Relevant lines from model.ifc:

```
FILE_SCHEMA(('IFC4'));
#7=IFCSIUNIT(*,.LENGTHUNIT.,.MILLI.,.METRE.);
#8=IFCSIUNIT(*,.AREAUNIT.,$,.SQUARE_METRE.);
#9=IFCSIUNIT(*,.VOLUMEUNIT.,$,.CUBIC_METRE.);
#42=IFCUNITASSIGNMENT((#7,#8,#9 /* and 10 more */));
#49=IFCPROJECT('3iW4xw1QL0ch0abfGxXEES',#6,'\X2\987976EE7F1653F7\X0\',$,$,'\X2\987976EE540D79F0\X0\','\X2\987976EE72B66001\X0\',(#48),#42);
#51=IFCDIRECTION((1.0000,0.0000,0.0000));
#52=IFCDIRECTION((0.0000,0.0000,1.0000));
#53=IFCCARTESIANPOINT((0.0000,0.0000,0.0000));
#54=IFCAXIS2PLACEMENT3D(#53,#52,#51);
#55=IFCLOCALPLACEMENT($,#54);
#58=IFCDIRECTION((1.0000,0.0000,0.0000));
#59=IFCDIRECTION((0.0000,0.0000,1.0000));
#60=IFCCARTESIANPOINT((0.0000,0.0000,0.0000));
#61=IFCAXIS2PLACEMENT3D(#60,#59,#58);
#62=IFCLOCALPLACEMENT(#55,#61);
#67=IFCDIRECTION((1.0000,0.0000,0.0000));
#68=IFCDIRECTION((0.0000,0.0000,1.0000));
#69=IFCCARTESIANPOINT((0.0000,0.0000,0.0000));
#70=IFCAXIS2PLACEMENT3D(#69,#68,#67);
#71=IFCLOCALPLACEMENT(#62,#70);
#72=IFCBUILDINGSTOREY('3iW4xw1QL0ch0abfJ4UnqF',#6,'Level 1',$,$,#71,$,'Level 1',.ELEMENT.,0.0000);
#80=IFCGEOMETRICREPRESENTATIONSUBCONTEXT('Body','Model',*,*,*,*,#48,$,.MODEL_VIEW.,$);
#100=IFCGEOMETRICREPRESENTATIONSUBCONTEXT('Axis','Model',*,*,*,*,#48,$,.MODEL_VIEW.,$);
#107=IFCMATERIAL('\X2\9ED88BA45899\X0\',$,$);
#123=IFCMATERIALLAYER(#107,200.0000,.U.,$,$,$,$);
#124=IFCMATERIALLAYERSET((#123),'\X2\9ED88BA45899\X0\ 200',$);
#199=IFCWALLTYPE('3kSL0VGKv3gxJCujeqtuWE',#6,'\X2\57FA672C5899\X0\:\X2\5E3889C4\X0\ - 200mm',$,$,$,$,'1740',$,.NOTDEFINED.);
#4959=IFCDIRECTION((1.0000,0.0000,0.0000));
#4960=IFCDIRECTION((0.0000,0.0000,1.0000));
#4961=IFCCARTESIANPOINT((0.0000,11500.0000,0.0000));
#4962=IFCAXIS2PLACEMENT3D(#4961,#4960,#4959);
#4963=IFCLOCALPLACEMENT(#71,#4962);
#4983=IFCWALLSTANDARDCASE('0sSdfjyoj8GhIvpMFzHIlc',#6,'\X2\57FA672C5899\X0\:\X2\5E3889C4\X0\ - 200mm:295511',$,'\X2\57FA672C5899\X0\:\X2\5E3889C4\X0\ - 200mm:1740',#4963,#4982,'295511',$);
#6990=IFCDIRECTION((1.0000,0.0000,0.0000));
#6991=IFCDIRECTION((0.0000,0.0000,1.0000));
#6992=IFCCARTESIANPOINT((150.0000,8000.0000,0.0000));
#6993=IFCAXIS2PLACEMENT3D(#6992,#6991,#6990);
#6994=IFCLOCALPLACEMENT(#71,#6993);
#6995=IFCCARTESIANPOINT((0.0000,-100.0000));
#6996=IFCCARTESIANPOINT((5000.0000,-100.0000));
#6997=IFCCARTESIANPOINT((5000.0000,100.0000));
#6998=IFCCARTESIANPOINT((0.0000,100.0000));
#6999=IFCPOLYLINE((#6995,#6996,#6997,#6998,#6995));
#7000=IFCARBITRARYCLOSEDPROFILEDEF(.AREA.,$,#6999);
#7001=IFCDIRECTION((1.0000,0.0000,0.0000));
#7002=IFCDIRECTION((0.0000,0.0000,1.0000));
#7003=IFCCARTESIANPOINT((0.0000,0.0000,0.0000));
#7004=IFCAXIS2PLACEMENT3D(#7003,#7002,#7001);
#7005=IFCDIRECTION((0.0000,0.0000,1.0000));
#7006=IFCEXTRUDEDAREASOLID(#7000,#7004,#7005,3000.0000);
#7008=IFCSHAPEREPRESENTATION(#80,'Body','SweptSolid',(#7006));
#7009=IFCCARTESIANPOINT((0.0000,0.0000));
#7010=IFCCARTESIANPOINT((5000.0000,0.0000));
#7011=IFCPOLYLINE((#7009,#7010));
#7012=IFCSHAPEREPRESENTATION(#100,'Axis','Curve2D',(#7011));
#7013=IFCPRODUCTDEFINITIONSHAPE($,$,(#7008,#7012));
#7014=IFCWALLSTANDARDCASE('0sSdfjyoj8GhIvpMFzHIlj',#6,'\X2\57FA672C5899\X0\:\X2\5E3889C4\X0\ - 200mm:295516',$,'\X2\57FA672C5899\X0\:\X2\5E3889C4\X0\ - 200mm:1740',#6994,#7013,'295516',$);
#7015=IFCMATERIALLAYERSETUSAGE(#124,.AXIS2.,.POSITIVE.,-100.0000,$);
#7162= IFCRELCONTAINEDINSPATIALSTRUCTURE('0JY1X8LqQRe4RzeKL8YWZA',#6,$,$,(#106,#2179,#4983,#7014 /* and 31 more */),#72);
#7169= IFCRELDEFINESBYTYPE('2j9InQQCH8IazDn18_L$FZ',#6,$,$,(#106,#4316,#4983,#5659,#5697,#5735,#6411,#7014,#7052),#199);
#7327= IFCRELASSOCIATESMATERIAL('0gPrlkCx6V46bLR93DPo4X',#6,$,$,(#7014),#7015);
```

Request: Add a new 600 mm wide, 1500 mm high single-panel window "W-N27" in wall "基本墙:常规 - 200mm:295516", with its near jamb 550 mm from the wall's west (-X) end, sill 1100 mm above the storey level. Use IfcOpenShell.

```python
import numpy as np
import ifcopenshell
import ifcopenshell.api.feature
import ifcopenshell.api.geometry
import ifcopenshell.api.root
import ifcopenshell.api.spatial
import ifcopenshell.geom
import ifcopenshell.util.element
import ifcopenshell.util.placement
import ifcopenshell.util.representation
import ifcopenshell.util.shape
import ifcopenshell.util.unit

model = ifcopenshell.open("model.ifc")
unit_scale = ifcopenshell.util.unit.calculate_unit_scale(model)
settings = ifcopenshell.geom.settings()


def volume(element):
    """Net volume in cubic metres, openings subtracted."""
    shape = ifcopenshell.geom.create_shape(settings, element)
    return ifcopenshell.util.shape.get_volume(shape.geometry)


wall = model.by_id(7014)
storey = ifcopenshell.util.element.get_container(wall, ifc_class="IfcBuildingStorey")
context = ifcopenshell.util.representation.get_context(model, "Model", "Body", "MODEL_VIEW")
before = volume(wall)

width, height, from_end, sill = 0.6, 1.5, 0.55, 1.1  # metres

# The wall runs along its own X axis, and the end named is its -X end.
wall_shape = ifcopenshell.geom.create_shape(settings, wall)
x, y, z = ifcopenshell.util.shape.get_vertices(wall_shape.geometry).T
start = x.min() + from_end
face, thickness = float(y.min()), float(y.max() - y.min())
wall_matrix = ifcopenshell.util.placement.get_local_placement(wall.ObjectPlacement)
level = ifcopenshell.util.placement.get_local_placement(storey.ObjectPlacement)[2, 3]


def in_wall(x, y):
    """Placement at x, y metres in the wall's axes, at sill height."""
    matrix = wall_matrix.copy()
    matrix[:, 3] = wall_matrix @ np.array([x / unit_scale, y / unit_scale, 0.0, 1.0])
    matrix[2, 3] = level + sill / unit_scale
    return matrix


# Opening: a box that overshoots both wall faces by 50 mm.
opening = ifcopenshell.api.root.create_entity(model, ifc_class="IfcOpeningElement", predefined_type="OPENING")
box = ifcopenshell.api.geometry.add_wall_representation(
    model, context=context, length=width, height=height, thickness=thickness + 0.1
)
ifcopenshell.api.geometry.assign_representation(model, product=opening, representation=box)
ifcopenshell.api.geometry.edit_object_placement(model, product=opening, matrix=in_wall(start, face - 0.05), is_si=False)
ifcopenshell.api.feature.add_feature(model, feature=opening, element=wall)

window = ifcopenshell.api.root.create_entity(model, ifc_class="IfcWindow", name="W-N27", predefined_type="WINDOW")
window.OverallWidth, window.OverallHeight = width / unit_scale, height / unit_scale
window.PartitioningType = "SINGLE_PANEL"
body = ifcopenshell.api.geometry.add_window_representation(
    model,
    context=context,
    overall_width=window.OverallWidth,
    overall_height=window.OverallHeight,
    partition_type="SINGLE_PANEL",
)
ifcopenshell.api.geometry.assign_representation(model, product=window, representation=body)
ifcopenshell.api.spatial.assign_container(model, products=[window], relating_structure=storey)
ifcopenshell.api.feature.add_filling(model, opening=opening, element=window)

# Centre the window in the wall's thickness.
ifcopenshell.api.geometry.edit_object_placement(model, product=window, matrix=in_wall(start, face), is_si=False)
window_shape = ifcopenshell.geom.create_shape(settings, window)
depth = ifcopenshell.util.shape.get_vertices(window_shape.geometry)[:, 1]
offset = face + thickness / 2 - (depth.min() + depth.max()) / 2
ifcopenshell.api.geometry.edit_object_placement(model, product=window, matrix=in_wall(start, offset), is_si=False)

after = volume(wall)

print(f"wall volume {before:.3f} -> {after:.3f} m3")

model.write("model_edited.ifc")
```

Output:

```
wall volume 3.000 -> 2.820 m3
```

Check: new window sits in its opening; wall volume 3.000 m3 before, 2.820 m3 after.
